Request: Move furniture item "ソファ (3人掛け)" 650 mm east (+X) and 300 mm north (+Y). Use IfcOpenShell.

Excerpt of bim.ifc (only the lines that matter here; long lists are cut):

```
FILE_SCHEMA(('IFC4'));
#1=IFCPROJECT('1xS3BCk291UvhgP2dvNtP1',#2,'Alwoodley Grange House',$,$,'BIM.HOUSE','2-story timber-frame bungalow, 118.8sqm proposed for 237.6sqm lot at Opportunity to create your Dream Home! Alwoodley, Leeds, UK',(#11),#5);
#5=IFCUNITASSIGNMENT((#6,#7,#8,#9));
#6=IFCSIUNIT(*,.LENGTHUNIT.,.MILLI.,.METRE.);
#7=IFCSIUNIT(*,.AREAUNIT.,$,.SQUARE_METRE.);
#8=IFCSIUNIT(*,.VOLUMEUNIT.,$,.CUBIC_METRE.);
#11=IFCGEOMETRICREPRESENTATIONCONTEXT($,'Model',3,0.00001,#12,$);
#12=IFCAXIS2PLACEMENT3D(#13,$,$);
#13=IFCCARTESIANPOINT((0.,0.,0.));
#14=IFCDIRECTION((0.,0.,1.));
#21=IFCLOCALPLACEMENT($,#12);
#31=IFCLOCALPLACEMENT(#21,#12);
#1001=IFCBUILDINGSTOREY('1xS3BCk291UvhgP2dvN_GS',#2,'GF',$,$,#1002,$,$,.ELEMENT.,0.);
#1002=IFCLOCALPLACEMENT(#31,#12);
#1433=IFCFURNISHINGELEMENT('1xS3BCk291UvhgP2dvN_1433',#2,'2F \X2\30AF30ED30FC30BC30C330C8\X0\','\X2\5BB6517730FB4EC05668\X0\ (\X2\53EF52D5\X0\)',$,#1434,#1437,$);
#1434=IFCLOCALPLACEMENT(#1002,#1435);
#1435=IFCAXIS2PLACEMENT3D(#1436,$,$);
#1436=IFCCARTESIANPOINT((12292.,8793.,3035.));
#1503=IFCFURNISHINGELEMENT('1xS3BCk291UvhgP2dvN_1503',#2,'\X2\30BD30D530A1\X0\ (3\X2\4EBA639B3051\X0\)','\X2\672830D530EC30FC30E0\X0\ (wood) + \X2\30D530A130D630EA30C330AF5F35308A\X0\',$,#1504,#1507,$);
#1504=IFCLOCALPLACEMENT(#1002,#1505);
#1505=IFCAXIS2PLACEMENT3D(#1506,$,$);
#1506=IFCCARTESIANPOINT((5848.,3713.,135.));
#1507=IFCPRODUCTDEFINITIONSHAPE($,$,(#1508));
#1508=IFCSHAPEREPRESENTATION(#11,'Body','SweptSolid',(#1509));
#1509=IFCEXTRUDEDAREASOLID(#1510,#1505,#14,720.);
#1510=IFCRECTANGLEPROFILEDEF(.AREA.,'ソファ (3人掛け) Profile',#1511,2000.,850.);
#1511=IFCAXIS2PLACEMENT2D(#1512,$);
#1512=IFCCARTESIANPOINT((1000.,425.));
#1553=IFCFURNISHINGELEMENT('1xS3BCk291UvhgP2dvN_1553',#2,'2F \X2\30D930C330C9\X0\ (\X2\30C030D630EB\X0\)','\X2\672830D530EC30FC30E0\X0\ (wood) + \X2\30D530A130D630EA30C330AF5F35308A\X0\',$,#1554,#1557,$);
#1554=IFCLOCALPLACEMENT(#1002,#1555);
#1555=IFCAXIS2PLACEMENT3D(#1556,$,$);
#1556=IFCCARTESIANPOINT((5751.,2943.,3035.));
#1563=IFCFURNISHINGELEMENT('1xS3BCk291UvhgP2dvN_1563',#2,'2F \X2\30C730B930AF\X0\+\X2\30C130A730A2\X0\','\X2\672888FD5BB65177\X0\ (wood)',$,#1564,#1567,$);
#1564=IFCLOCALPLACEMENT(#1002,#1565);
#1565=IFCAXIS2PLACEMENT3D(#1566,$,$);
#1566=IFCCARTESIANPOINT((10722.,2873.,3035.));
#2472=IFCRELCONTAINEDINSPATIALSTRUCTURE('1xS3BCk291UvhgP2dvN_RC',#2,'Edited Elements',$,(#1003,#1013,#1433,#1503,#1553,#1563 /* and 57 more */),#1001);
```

```python
import ifcopenshell
import ifcopenshell.api.geometry
import ifcopenshell.util.placement
import ifcopenshell.util.unit

model = ifcopenshell.open("bim.ifc")
unit_scale = ifcopenshell.util.unit.calculate_unit_scale(model)

item = model.by_guid("1xS3BCk291UvhgP2dvN_1503")
matrix = ifcopenshell.util.placement.get_local_placement(item.ObjectPlacement)
matrix[0, 3] += 0.65 / unit_scale
matrix[1, 3] += 0.3 / unit_scale
ifcopenshell.api.geometry.edit_object_placement(model, product=item, matrix=matrix, is_si=False)

print(ifcopenshell.util.placement.get_local_placement(item.ObjectPlacement).round(3) + 0.0)

model.write("bim_edited.ifc")
```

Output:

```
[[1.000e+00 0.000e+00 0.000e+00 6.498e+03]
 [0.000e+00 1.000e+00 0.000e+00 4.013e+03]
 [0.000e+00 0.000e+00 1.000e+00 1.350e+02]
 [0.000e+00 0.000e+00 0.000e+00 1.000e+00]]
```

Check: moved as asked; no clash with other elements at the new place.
